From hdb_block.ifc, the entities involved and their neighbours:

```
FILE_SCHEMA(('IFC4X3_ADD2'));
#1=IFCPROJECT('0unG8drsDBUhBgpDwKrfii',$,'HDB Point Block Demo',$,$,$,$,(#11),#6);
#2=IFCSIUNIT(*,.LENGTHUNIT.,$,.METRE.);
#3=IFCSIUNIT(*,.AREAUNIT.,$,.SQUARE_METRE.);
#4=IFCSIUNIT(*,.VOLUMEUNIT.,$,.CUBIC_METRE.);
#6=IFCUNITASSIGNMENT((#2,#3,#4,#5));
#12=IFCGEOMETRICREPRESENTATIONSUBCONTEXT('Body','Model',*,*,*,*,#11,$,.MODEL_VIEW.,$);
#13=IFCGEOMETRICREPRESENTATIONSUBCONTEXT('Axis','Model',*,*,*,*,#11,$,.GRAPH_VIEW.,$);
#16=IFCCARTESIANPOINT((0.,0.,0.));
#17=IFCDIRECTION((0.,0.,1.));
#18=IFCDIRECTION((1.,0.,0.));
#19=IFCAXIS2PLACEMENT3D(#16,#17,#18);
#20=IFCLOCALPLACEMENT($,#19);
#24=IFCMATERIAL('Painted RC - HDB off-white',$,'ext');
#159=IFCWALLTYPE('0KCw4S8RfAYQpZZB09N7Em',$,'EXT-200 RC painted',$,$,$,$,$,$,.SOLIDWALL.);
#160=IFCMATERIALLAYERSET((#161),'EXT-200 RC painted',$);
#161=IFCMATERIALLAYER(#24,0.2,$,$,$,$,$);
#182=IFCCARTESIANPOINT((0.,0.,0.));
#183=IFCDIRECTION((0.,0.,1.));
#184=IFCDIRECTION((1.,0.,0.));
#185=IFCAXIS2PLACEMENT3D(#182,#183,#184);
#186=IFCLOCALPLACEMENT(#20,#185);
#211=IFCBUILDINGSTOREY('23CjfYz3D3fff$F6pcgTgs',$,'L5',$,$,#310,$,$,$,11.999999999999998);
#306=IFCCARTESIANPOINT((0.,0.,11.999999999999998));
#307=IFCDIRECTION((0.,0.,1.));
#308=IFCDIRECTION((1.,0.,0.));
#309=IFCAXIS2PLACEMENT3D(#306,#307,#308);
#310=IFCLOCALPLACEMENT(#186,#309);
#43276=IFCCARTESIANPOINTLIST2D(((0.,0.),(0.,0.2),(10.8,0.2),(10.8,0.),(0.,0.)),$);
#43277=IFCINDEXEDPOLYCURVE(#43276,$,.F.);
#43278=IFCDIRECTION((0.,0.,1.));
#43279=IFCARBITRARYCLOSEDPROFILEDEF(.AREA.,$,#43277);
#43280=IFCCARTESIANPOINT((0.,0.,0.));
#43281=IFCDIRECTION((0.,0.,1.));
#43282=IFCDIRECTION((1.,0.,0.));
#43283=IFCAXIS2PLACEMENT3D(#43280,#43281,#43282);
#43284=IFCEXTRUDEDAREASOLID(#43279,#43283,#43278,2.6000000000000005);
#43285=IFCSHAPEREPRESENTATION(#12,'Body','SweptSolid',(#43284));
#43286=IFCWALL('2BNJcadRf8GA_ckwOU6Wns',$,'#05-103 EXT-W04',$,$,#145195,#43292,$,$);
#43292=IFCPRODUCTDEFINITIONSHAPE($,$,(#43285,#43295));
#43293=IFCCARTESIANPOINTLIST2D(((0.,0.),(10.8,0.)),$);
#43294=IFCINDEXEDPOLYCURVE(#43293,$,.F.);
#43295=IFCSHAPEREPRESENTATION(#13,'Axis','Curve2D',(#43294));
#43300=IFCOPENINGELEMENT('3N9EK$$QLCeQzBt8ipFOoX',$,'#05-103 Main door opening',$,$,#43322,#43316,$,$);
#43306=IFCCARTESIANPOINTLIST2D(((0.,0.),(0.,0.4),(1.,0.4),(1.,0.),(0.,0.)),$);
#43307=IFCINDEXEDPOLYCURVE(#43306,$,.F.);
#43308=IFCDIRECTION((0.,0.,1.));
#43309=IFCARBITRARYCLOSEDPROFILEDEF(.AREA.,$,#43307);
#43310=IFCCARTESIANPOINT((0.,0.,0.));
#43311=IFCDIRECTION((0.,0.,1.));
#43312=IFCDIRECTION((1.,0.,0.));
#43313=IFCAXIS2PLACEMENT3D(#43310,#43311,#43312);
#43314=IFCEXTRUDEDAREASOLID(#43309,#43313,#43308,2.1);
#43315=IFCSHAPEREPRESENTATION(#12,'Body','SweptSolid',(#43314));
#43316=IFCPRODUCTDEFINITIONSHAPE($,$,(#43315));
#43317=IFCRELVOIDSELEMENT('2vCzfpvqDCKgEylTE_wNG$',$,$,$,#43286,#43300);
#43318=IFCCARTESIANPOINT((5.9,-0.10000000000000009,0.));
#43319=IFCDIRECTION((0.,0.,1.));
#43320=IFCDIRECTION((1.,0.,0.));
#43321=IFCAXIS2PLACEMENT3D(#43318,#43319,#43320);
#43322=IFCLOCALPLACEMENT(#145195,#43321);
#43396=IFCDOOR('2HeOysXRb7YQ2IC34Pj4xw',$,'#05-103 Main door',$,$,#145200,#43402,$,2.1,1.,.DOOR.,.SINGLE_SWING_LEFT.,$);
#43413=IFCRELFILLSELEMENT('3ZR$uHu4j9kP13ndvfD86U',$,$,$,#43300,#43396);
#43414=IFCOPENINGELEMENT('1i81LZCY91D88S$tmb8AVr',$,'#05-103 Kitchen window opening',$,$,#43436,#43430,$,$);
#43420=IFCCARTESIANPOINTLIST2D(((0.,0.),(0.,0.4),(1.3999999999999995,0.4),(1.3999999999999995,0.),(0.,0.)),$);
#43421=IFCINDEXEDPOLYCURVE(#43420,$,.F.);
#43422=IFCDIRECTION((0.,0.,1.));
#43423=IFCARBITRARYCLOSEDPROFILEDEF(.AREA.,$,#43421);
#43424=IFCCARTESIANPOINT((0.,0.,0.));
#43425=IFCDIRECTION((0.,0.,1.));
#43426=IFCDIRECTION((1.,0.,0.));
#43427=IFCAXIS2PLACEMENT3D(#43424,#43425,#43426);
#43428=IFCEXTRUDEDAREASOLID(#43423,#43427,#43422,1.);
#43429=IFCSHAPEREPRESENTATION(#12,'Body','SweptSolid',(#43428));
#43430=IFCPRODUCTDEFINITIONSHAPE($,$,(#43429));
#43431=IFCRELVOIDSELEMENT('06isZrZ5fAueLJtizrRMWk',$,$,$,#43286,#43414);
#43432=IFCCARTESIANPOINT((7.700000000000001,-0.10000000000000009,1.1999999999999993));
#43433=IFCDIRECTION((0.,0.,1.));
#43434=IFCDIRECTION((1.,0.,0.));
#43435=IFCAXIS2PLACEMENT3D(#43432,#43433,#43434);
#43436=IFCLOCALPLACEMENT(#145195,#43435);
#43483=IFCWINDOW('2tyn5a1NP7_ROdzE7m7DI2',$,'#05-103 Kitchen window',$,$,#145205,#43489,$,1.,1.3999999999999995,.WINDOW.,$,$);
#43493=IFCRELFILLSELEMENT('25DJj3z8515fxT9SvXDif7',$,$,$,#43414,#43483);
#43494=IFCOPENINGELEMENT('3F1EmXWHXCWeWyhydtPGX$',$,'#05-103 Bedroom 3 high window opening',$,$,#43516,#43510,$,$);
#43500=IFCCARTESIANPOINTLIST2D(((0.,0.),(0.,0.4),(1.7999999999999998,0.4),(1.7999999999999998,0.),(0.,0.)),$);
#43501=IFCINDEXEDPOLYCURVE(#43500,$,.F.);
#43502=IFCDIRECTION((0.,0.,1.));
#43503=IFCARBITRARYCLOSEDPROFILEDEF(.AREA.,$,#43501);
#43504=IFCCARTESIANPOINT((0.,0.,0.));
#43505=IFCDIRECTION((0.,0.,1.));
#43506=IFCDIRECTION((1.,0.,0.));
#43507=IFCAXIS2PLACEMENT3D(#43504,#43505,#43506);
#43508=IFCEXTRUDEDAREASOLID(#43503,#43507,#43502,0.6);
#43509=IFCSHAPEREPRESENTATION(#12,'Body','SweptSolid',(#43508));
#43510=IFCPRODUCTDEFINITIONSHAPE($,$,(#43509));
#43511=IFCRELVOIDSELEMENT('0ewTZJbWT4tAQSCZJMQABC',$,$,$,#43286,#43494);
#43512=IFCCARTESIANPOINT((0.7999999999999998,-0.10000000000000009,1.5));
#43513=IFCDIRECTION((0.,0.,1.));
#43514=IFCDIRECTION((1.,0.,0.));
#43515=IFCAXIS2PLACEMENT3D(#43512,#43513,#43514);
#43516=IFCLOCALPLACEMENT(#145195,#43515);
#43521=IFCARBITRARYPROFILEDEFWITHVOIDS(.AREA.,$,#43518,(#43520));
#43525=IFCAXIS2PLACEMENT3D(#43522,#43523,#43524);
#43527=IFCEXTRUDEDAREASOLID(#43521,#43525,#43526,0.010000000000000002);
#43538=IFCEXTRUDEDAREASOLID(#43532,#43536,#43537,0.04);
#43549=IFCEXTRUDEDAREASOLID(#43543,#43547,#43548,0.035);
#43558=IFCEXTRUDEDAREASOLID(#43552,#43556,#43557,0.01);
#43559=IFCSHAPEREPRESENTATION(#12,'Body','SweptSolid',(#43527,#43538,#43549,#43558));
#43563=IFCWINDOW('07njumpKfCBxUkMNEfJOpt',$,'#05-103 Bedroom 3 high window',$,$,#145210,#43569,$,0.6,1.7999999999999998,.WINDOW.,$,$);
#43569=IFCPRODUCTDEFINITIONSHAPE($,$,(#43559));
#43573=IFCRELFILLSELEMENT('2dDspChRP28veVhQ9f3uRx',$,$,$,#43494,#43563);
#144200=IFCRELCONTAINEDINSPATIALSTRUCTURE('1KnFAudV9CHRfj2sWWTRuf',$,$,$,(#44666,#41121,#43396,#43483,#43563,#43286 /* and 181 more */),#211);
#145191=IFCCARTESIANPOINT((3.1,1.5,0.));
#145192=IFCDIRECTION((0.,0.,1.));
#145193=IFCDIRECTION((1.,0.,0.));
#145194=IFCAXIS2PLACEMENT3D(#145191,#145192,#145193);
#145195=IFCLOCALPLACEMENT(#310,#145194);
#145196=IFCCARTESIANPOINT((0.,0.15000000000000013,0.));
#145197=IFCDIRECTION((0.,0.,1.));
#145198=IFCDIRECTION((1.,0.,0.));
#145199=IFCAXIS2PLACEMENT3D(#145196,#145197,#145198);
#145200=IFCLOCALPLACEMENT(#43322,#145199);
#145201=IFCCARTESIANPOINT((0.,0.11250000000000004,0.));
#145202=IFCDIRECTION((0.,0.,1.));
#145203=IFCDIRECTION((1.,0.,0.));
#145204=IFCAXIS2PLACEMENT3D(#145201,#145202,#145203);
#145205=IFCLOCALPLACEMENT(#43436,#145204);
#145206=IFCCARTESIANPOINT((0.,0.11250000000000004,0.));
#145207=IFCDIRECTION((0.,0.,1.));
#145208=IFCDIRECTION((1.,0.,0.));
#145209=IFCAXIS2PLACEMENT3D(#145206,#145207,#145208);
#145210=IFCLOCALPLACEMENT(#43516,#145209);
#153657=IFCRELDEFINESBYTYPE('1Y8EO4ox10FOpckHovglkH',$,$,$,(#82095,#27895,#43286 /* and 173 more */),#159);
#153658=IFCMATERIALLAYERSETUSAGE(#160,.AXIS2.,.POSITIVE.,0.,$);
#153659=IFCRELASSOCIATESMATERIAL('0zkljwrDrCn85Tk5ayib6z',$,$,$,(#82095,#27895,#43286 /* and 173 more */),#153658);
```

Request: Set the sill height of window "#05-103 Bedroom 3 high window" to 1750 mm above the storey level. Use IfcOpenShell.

```python
import numpy as np
import ifcopenshell
import ifcopenshell.api.geometry
import ifcopenshell.geom
import ifcopenshell.util.element
import ifcopenshell.util.placement
import ifcopenshell.util.shape
import ifcopenshell.util.unit

model = ifcopenshell.open("hdb_block.ifc")
unit_scale = ifcopenshell.util.unit.calculate_unit_scale(model)

window = model.by_id(43563)
opening = window.FillsVoids[0].RelatingOpeningElement
storey = ifcopenshell.util.element.get_container(window, ifc_class="IfcBuildingStorey")
level = ifcopenshell.util.placement.get_local_placement(storey.ObjectPlacement)[2, 3]

# The opening's origin need not be at the sill, so measure its lowest point.
shape = ifcopenshell.geom.create_shape(ifcopenshell.geom.settings(), opening)
bottom = ifcopenshell.util.shape.get_shape_bottom_elevation(shape, shape.geometry) / unit_scale
dz = level + 1.75 / unit_scale - bottom

shift = np.array([0.0, 0.0, dz])
# The window is placed relative to its opening, so it follows when the opening moves.
matrix = ifcopenshell.util.placement.get_local_placement(opening.ObjectPlacement)
matrix[:3, 3] += shift
ifcopenshell.api.geometry.edit_object_placement(
    model, product=opening, matrix=matrix, is_si=False, should_transform_children=True
)

print(f"moved by {dz * unit_scale:+.3f} m")

model.write("hdb_block_v2.ifc")
```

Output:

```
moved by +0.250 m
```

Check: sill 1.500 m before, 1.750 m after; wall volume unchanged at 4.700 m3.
